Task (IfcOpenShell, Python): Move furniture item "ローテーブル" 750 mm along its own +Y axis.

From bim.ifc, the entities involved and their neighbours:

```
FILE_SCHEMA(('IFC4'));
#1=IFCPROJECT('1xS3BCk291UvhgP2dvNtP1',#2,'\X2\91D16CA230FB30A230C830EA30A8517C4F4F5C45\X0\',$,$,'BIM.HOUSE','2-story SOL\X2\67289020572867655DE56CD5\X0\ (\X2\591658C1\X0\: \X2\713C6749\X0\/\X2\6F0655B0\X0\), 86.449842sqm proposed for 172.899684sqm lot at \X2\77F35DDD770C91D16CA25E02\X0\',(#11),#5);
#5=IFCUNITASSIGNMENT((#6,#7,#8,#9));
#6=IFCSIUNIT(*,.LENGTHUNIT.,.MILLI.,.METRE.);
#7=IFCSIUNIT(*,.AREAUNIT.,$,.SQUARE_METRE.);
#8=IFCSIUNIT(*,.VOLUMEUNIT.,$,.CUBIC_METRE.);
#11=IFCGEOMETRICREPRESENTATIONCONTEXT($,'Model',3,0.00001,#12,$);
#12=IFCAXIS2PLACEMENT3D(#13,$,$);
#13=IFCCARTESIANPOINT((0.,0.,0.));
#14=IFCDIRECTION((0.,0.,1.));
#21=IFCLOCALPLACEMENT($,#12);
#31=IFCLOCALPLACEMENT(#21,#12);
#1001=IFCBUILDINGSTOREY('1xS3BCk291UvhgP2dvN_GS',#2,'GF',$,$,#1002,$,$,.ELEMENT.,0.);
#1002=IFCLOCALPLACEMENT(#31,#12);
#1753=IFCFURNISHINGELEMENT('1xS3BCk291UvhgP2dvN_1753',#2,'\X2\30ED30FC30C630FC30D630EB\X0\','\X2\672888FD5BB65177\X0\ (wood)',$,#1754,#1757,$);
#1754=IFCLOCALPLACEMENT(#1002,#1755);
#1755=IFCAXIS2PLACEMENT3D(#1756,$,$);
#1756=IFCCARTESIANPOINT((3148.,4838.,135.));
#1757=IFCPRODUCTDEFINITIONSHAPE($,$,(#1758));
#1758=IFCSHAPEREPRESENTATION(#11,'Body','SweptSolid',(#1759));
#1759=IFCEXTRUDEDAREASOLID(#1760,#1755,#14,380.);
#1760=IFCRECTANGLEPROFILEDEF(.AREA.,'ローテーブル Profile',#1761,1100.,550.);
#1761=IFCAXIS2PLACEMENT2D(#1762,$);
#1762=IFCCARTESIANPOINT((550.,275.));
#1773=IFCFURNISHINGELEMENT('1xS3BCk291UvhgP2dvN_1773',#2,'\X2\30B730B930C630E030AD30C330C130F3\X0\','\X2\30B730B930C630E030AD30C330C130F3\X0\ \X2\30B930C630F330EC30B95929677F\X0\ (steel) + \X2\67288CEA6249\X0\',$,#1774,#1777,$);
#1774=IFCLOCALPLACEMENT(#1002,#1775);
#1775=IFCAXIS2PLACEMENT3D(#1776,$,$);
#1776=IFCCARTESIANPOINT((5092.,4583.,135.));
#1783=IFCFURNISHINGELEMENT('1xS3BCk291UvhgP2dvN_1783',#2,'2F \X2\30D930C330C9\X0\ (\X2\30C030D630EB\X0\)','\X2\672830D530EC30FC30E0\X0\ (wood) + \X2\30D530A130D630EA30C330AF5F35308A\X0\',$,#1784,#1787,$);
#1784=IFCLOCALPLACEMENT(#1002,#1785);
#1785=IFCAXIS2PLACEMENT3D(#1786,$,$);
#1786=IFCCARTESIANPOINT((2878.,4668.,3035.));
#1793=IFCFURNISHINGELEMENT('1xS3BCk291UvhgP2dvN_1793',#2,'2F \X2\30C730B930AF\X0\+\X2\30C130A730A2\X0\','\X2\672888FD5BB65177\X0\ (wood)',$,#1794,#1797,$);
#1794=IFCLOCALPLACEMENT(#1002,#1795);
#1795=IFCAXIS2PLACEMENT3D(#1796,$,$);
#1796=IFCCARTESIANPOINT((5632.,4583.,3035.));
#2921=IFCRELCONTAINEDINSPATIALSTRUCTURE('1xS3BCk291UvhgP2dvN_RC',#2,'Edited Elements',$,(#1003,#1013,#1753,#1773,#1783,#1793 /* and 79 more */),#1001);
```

```python
import ifcopenshell
import ifcopenshell.api.geometry
import ifcopenshell.util.placement
import ifcopenshell.util.unit

model = ifcopenshell.open("bim.ifc")
unit_scale = ifcopenshell.util.unit.calculate_unit_scale(model)

item = model.by_id(1753)
matrix = ifcopenshell.util.placement.get_local_placement(item.ObjectPlacement)
matrix[:3, 3] += matrix[:3, 1] * 0.75 / unit_scale
ifcopenshell.api.geometry.edit_object_placement(model, product=item, matrix=matrix, is_si=False)

print(ifcopenshell.util.placement.get_local_placement(item.ObjectPlacement).round(3) + 0.0)

model.write("bim-out.ifc")
```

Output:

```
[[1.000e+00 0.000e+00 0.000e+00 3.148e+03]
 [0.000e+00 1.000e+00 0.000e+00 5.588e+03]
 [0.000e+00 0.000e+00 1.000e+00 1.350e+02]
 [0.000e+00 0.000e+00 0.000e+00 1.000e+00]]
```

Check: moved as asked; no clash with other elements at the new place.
